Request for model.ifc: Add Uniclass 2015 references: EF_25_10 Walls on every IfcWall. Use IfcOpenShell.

First a look at what the model holds.

```python
import ifcopenshell

model = ifcopenshell.open("model.ifc")
print(model.schema)
print("classifications:", [c.Name for c in model.by_type("IfcClassification")])
for ifc_class in ("IfcDoor", "IfcRoof", "IfcStair", "IfcWall", "IfcWindow"):
    print(ifc_class, len(model.by_type(ifc_class)))
```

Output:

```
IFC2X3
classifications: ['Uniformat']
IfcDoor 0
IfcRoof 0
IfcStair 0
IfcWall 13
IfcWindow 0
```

```python
import ifcopenshell
import ifcopenshell.api.classification

model = ifcopenshell.open("model.ifc")

# IFC2X3 requires Source and Edition and has no link from the project to the system.
system = model.create_entity("IfcClassification", Source="NBS", Edition="2015", Name="Uniclass 2015")

codes = {
    "IfcWall": ("EF_25_10", "Walls"),
}
for ifc_class, (code, name) in codes.items():
    products = model.by_type(ifc_class)
    ifcopenshell.api.classification.add_reference(
        model, products=products, classification=system, identification=code, name=name
    )
    print(code, len(products))

model.write("model_rev.ifc")
```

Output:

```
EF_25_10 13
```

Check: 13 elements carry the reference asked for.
